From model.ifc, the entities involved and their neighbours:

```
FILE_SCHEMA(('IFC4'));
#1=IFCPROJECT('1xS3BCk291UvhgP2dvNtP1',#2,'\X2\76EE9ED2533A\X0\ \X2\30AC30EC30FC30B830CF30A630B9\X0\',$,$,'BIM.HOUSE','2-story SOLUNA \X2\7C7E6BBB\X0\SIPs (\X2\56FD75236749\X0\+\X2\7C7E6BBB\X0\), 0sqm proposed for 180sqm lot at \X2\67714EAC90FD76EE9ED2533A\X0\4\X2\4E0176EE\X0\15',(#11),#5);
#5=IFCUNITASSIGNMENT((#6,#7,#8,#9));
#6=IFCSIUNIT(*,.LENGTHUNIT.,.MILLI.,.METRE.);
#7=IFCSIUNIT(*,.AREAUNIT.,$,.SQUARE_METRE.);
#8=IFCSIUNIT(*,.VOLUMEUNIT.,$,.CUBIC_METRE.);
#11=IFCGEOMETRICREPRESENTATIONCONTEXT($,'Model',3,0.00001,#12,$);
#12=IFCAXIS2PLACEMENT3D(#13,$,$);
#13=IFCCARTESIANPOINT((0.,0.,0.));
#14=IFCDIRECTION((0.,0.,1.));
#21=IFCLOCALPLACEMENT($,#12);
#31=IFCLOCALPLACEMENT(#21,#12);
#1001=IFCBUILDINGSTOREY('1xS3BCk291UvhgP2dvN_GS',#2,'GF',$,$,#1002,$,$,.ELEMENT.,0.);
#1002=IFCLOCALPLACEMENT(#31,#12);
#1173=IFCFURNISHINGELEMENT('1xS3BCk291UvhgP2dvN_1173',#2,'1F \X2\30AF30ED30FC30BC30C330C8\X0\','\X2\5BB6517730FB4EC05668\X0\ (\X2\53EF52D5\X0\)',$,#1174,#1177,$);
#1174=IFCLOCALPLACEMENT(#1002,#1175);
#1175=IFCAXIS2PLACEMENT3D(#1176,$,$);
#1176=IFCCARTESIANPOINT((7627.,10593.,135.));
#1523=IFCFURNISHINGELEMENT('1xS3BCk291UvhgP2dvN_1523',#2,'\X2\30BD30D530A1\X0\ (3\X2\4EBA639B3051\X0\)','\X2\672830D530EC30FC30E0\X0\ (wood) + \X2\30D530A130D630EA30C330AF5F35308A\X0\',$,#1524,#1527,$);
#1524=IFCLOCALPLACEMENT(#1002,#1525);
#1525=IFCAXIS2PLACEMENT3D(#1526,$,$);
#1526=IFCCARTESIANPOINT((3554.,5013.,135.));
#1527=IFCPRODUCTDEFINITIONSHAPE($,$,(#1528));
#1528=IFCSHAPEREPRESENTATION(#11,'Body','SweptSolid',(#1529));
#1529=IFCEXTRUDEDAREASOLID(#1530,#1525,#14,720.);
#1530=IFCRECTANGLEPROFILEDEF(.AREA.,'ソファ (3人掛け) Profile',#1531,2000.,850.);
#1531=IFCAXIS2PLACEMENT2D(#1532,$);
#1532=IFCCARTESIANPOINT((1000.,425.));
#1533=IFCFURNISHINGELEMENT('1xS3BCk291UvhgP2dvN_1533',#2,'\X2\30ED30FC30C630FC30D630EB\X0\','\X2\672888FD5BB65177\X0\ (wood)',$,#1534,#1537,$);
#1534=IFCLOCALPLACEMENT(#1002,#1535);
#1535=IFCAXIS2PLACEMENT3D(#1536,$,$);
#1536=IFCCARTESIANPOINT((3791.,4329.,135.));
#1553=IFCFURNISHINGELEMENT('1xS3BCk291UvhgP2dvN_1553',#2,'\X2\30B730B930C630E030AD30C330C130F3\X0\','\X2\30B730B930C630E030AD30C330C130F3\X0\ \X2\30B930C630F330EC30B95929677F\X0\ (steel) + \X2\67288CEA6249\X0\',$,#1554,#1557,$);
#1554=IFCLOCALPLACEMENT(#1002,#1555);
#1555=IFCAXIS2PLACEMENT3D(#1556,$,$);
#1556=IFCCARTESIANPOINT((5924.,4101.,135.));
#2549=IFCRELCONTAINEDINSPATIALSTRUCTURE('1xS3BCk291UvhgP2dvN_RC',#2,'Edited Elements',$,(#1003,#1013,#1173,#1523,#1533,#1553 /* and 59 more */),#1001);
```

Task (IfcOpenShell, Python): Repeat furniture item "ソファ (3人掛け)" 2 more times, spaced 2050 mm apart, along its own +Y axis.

```python
import ifcopenshell
import ifcopenshell.api.geometry
import ifcopenshell.api.root
import ifcopenshell.util.element
import ifcopenshell.util.placement

model = ifcopenshell.open("model.ifc")


def reuse_history(source, copy):
    """copy_class also copies each property set's owner history, people and application; keep the originals."""
    for rel in copy.IsDefinedBy:
        if rel.is_a("IfcRelDefinesByProperties") and (history := rel.RelatingPropertyDefinition.OwnerHistory):
            rel.RelatingPropertyDefinition.OwnerHistory = source.OwnerHistory
            ifcopenshell.util.element.remove_deep2(model, history)


source = model.by_guid("1xS3BCk291UvhgP2dvN_1523")
base = ifcopenshell.util.placement.get_local_placement(source.ObjectPlacement)
step = base[:3, 1] * 2050.0

for i in range(1, 3):
    copy = ifcopenshell.api.root.copy_class(model, product=source)
    copy.Representation = ifcopenshell.util.element.copy_deep(
        model, source.Representation, exclude=["IfcGeometricRepresentationContext", "IfcRepresentationMap"]
    )
    reuse_history(source, copy)
    matrix = base.copy()
    matrix[:3, 3] += i * step
    print("added at", matrix[:3, 3].round(3) + 0.0)
    ifcopenshell.api.geometry.edit_object_placement(model, product=copy, matrix=matrix, is_si=False)

model.write("model_edited.ifc")
```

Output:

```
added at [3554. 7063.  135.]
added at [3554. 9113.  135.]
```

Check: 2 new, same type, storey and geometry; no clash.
